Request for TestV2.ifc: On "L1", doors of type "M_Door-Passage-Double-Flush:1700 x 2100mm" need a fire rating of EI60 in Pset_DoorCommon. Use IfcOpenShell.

First a look at what the model holds.

```python
import ifcopenshell
import ifcopenshell.util.element

model = ifcopenshell.open("TestV2.ifc")
print(model.schema)
storey = next(s for s in model.by_type("IfcBuildingStorey") if s.Name == "L1")
doors = [e for e in ifcopenshell.util.element.get_decomposition(storey) if e.is_a("IfcDoor")]
seen = {}
for e in doors:
    element_type = ifcopenshell.util.element.get_type(e)
    key = (element_type.Name if element_type != e and element_type else None, ifcopenshell.util.element.get_pset(e, "Pset_DoorCommon", "FireRating"))
    seen[key] = seen.get(key, 0) + 1
for (name, value), count in sorted(seen.items(), key=str):
    print(count, "x", name, "|", value)
```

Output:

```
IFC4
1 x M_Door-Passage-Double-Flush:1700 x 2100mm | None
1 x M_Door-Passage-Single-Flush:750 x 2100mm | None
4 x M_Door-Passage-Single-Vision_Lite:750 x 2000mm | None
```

```python
import ifcopenshell
import ifcopenshell.api.pset
import ifcopenshell.util.element

model = ifcopenshell.open("TestV2.ifc")

storey = next(s for s in model.by_type("IfcBuildingStorey") if s.Name == "L1")
doors = [e for e in ifcopenshell.util.element.get_decomposition(storey) if e.is_a("IfcDoor")]

count = 0
for e in doors:
    element_type = ifcopenshell.util.element.get_type(e)
    if element_type in (None, e) or element_type.Name != "M_Door-Passage-Double-Flush:1700 x 2100mm":
        continue
    # add_pset returns the element's existing set when there is one.
    pset = ifcopenshell.api.pset.add_pset(model, product=e, name="Pset_DoorCommon")
    ifcopenshell.api.pset.edit_pset(model, pset=pset, properties={"FireRating": "EI60"})
    count += 1

print(count, "doors updated")

model.write("TestV2_updated.ifc")
```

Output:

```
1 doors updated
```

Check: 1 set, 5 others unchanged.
